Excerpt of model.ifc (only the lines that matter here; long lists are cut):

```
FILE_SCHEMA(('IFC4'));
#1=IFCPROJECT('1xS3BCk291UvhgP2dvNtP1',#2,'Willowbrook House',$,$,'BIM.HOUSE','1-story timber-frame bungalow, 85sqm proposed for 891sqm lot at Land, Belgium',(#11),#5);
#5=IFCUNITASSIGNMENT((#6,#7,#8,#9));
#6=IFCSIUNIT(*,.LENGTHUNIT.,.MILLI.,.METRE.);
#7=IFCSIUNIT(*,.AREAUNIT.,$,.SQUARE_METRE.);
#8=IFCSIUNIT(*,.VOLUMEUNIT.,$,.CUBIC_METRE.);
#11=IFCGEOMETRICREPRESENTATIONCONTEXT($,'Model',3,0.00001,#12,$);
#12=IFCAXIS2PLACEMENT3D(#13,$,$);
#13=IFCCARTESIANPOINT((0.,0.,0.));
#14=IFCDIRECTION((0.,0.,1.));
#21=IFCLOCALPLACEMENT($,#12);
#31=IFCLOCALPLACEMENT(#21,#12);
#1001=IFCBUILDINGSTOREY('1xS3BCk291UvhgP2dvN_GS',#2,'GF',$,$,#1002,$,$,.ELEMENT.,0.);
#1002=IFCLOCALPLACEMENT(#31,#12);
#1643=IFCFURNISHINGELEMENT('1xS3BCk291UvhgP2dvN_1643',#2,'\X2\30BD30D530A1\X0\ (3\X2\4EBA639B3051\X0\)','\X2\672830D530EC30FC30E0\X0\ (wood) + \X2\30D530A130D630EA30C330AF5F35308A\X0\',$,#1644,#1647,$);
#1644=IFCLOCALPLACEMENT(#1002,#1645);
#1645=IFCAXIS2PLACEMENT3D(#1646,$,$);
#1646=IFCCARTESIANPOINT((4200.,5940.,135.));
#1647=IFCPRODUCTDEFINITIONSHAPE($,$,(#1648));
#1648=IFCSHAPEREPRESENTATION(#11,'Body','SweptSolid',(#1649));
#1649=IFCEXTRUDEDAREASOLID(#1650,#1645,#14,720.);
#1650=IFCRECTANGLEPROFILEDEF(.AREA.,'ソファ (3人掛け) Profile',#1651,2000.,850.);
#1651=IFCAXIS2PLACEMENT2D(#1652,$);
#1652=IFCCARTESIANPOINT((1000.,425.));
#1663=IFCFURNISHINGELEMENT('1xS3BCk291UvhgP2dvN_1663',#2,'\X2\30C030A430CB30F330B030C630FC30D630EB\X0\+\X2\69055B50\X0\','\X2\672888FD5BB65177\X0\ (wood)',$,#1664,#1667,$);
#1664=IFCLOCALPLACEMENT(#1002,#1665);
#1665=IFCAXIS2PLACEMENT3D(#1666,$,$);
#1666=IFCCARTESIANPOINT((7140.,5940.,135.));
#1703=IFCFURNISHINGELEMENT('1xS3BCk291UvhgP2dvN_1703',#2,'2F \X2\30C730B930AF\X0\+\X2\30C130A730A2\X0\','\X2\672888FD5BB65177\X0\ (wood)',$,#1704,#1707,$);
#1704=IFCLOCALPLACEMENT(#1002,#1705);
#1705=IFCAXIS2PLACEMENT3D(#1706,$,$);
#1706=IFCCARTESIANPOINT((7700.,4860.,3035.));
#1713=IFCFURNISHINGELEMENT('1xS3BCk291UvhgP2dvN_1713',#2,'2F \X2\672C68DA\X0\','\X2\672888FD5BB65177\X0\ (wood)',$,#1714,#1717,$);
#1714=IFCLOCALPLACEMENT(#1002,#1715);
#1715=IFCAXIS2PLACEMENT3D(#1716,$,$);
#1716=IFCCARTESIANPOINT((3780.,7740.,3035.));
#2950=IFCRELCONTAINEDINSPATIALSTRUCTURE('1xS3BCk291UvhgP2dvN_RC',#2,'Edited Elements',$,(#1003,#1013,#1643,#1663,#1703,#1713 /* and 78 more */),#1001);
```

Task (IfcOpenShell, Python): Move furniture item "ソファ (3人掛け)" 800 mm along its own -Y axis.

```python
import ifcopenshell
import ifcopenshell.api.geometry
import ifcopenshell.util.placement

model = ifcopenshell.open("model.ifc")

item = model.by_guid("1xS3BCk291UvhgP2dvN_1643")
matrix = ifcopenshell.util.placement.get_local_placement(item.ObjectPlacement)
matrix[:3, 3] -= matrix[:3, 1] * 800.0
ifcopenshell.api.geometry.edit_object_placement(model, product=item, matrix=matrix, is_si=False)

print(ifcopenshell.util.placement.get_local_placement(item.ObjectPlacement).round(3) + 0.0)

model.write("model_v2.ifc")
```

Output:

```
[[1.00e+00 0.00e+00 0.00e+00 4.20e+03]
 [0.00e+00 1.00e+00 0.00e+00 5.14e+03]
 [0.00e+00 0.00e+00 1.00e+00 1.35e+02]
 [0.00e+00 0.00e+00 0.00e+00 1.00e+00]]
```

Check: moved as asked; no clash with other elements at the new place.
